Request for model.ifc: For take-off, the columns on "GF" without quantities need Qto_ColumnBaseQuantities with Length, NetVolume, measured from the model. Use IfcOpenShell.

First a look at what the model holds.

```python
import ifcopenshell
import ifcopenshell.util.element
import ifcopenshell.util.unit

model = ifcopenshell.open("model.ifc")
print(model.schema)
for unit_type in ("LENGTHUNIT", "AREAUNIT", "VOLUMEUNIT"):
    print(unit_type, ifcopenshell.util.unit.calculate_unit_scale(model, unit_type))
storey = next(s for s in model.by_type("IfcBuildingStorey") if s.Name == "GF")
columns = [e for e in ifcopenshell.util.element.get_decomposition(storey) if e.is_a("IfcColumn")]
for e in sorted(columns, key=lambda e: e.id()):
    print(e.id(), e.is_a(), e.Name, list(ifcopenshell.util.element.get_psets(e, qtos_only=True)), sep=" | ")
```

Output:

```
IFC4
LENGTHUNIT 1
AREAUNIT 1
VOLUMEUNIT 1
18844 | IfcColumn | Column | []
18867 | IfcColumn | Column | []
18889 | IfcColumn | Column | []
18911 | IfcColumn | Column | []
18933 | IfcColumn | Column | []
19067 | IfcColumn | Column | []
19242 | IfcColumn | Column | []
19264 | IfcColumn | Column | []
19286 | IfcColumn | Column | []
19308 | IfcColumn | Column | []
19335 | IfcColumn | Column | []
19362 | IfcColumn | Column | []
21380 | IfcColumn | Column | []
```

```python
import ifcopenshell
import ifcopenshell.api.pset
import ifcopenshell.geom
import ifcopenshell.util.element
import ifcopenshell.util.shape
import ifcopenshell.util.unit

model = ifcopenshell.open("model.ifc")
unit_scale = ifcopenshell.util.unit.calculate_unit_scale(model)
volume_scale = ifcopenshell.util.unit.calculate_unit_scale(model, "VOLUMEUNIT")
settings = ifcopenshell.geom.settings()

storey = next(s for s in model.by_type("IfcBuildingStorey") if s.Name == "GF")
columns = [e for e in ifcopenshell.util.element.get_decomposition(storey) if e.is_a("IfcColumn")]

for e in sorted(columns, key=lambda e: e.id()):
    if ifcopenshell.util.element.get_psets(e, qtos_only=True, should_inherit=False):
        continue
    # Geometry comes back in metres, in the element's own axes.
    shape = ifcopenshell.geom.create_shape(settings, e)
    values = {
        "Length": ifcopenshell.util.shape.get_z(shape.geometry) / unit_scale,
        "NetVolume": ifcopenshell.util.shape.get_volume(shape.geometry) / volume_scale,
    }
    qto = ifcopenshell.api.pset.add_qto(model, product=e, name="Qto_ColumnBaseQuantities")
    ifcopenshell.api.pset.edit_qto(model, qto=qto, properties=values)
    print(e.id(), {k: round(v, 3) for k, v in values.items()})

model.write("model_v2.ifc")
```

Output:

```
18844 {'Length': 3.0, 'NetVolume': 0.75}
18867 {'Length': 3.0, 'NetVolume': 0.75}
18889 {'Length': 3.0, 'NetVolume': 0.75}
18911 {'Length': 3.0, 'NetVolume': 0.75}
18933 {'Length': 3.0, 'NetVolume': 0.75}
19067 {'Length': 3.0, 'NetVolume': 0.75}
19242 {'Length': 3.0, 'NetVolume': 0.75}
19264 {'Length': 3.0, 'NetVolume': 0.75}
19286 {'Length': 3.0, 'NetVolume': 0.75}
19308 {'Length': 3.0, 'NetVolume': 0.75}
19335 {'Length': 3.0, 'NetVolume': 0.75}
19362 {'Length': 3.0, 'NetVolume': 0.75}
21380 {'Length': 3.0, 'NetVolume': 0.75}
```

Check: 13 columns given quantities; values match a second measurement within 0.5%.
